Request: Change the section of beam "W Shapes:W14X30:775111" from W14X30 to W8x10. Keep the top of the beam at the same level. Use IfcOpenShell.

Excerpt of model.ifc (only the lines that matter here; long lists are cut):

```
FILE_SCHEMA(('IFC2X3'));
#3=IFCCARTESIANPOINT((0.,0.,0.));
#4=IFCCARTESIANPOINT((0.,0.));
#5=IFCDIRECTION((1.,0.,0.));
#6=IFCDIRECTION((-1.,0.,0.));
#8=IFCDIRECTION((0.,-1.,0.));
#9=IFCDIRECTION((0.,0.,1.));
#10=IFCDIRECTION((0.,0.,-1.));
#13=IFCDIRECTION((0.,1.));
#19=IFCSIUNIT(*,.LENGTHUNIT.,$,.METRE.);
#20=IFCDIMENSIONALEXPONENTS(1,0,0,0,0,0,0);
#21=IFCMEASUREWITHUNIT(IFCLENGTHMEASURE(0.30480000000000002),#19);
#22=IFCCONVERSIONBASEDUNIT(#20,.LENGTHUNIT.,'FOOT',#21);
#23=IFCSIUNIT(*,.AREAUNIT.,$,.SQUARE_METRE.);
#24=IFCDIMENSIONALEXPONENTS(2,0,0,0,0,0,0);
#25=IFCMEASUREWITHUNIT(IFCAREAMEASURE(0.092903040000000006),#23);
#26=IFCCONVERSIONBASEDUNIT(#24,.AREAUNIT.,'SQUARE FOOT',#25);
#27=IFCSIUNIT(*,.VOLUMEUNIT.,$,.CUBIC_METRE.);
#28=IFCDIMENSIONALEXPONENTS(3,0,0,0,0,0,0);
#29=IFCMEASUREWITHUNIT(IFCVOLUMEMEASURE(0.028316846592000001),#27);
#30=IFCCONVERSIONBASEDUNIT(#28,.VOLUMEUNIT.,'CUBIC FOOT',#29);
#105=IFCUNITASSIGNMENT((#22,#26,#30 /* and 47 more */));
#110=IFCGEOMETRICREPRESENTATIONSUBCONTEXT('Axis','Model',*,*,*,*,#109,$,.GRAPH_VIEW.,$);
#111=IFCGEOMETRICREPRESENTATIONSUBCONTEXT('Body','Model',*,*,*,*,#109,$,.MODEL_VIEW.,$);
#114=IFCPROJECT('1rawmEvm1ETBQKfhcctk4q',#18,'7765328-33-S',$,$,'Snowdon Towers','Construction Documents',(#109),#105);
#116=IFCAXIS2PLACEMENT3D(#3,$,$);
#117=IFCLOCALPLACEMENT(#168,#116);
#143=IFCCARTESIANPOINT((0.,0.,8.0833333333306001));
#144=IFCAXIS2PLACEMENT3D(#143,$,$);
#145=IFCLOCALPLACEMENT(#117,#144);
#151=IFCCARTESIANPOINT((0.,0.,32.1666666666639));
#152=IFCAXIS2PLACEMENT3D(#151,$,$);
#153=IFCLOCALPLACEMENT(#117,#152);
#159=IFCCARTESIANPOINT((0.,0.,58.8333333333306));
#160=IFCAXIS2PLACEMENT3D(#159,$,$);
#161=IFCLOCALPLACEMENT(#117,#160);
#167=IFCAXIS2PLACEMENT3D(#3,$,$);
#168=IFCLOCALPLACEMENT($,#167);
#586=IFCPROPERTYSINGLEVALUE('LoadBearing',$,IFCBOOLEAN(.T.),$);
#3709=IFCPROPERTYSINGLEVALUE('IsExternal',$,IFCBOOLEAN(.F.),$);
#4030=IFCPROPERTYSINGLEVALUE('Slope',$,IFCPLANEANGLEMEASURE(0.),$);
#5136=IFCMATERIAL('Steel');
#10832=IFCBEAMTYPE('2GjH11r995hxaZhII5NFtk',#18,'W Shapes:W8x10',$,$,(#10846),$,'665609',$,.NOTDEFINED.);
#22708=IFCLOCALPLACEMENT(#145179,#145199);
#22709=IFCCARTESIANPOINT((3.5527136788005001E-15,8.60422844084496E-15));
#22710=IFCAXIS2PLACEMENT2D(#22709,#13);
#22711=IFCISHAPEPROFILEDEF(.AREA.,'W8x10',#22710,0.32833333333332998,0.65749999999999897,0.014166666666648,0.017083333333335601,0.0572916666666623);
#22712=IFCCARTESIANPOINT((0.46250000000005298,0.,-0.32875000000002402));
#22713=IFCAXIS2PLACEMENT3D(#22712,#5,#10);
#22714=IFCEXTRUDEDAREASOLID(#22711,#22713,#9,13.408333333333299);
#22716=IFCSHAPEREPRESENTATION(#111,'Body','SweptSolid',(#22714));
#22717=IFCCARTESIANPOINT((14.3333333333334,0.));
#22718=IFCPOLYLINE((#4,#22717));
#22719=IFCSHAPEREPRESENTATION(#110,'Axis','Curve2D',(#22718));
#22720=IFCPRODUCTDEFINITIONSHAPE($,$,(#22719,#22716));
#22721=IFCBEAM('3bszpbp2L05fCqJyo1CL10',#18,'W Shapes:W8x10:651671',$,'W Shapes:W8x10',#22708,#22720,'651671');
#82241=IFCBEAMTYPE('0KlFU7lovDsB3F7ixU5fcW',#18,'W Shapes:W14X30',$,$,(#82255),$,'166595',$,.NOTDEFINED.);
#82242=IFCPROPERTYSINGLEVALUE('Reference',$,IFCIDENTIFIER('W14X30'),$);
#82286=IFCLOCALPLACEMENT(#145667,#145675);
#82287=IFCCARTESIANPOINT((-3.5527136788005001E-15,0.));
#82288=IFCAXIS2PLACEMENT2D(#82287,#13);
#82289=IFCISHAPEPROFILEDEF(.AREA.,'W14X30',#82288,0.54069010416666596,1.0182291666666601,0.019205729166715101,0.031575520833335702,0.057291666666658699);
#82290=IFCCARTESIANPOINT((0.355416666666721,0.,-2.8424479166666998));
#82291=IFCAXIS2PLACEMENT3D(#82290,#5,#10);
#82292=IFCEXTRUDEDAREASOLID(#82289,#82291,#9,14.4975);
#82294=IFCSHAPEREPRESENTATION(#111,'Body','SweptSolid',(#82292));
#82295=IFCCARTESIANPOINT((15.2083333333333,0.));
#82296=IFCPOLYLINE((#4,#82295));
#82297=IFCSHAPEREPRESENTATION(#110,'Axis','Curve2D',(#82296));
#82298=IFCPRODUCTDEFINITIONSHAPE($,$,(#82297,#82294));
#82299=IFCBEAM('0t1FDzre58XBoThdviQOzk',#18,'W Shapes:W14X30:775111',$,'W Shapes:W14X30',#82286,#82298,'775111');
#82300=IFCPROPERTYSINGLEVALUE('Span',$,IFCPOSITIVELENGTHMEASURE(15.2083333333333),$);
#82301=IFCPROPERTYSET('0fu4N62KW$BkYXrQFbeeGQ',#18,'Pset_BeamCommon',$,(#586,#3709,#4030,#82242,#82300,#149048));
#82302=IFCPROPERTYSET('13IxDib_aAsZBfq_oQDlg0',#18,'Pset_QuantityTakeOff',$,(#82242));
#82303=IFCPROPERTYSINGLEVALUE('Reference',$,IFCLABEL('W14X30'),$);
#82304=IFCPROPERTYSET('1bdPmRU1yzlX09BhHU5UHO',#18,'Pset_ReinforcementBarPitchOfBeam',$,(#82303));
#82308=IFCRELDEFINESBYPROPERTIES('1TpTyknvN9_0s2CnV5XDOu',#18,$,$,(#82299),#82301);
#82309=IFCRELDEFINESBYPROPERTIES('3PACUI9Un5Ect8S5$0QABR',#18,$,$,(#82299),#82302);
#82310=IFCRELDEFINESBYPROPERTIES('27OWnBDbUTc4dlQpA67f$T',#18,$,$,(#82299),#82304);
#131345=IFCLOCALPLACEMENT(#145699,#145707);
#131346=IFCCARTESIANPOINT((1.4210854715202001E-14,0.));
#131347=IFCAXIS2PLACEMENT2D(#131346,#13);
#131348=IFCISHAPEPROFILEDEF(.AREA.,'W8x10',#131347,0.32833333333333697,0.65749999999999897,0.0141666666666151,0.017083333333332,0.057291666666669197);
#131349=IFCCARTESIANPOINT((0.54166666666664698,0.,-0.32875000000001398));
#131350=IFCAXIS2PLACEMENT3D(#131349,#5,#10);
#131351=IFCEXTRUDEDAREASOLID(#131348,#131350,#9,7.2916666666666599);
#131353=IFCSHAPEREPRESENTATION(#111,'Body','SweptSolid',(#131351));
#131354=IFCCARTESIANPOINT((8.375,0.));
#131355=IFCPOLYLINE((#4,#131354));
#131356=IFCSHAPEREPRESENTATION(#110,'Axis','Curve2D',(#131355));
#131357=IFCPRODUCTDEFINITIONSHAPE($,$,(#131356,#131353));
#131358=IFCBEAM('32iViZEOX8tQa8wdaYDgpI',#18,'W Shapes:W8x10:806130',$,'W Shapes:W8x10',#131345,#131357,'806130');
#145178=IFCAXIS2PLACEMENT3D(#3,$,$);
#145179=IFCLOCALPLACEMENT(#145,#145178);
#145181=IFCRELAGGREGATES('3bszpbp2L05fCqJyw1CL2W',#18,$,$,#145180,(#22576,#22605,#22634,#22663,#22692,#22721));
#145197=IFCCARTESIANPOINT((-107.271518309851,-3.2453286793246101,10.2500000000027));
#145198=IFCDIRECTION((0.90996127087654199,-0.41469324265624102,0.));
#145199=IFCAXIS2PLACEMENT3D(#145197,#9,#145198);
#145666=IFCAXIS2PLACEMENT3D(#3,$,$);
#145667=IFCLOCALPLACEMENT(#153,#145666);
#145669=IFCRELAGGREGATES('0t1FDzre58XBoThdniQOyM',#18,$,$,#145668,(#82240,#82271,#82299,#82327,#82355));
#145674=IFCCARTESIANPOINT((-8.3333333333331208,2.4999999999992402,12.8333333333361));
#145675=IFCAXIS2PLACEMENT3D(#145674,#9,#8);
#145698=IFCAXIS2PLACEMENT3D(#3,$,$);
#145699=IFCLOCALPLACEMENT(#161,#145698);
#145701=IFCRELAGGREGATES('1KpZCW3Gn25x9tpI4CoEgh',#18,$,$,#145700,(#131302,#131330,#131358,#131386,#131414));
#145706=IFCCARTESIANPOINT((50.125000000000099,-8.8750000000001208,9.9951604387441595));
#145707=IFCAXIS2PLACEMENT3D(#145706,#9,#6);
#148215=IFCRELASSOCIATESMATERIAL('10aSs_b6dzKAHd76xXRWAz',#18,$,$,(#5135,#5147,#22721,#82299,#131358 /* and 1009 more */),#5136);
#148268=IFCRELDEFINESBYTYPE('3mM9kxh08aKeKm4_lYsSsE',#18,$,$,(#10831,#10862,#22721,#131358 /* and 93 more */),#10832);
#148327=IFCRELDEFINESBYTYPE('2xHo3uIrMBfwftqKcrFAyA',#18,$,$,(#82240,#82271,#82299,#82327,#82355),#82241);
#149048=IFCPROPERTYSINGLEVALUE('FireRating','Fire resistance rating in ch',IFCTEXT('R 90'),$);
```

```python
import ifcopenshell
import ifcopenshell.api.pset
import ifcopenshell.api.type
import ifcopenshell.util.element
import ifcopenshell.util.representation

model = ifcopenshell.open("model.ifc")

member = model.by_guid("0t1FDzre58XBoThdviQOzk")
source = next(p for p in model.by_type("IfcIShapeProfileDef") if p.ProfileName == "W8x10")

body = ifcopenshell.util.representation.get_representation(member, "Model", "Body")
solid = body.Items[0]
old_profile = solid.SweptArea

# Copy the section's sizes but keep this member's own profile position.
profile = ifcopenshell.util.element.copy(model, source)
# Profiles are centred, so shift by half the change in depth to hold the top.
shift = (old_profile.OverallDepth - profile.OverallDepth) / 2
x, y = old_profile.Position.Location.Coordinates
up = (-1.0, 0.0)  # upwards, in the solid's own plane
location = model.createIfcCartesianPoint((x + up[0] * shift, y + up[1] * shift))
profile.Position = model.createIfcAxis2Placement2D(location, old_profile.Position.RefDirection)
solid.SweptArea = profile
if not model.get_total_inverses(old_profile):
    ifcopenshell.util.element.remove_deep2(model, old_profile)

new_type = model.by_id(10832)
ifcopenshell.api.type.assign_type(
    model, related_objects=[member], relating_type=new_type, should_map_representations=False
)
member.Name = member.Name.replace("W14X30", "W8x10")
member.ObjectType = "W Shapes:W8x10"
pset = model.by_id(ifcopenshell.util.element.get_pset(member, "Pset_BeamCommon", should_inherit=False)["id"])
ifcopenshell.api.pset.edit_pset(model, pset=pset, properties={"Reference": "W8x10"})
pset = model.by_id(ifcopenshell.util.element.get_pset(member, "Pset_QuantityTakeOff", should_inherit=False)["id"])
ifcopenshell.api.pset.edit_pset(model, pset=pset, properties={"Reference": "W8x10"})
pset = model.by_id(ifcopenshell.util.element.get_pset(member, "Pset_ReinforcementBarPitchOfBeam", should_inherit=False)["id"])
ifcopenshell.api.pset.edit_pset(model, pset=pset, properties={"Reference": "W8x10"})

print(solid.SweptArea)

model.write("model_rev.ifc")
```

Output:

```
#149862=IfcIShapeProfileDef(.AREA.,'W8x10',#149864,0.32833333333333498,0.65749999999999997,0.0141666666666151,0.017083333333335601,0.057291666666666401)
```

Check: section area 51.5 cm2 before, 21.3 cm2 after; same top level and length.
